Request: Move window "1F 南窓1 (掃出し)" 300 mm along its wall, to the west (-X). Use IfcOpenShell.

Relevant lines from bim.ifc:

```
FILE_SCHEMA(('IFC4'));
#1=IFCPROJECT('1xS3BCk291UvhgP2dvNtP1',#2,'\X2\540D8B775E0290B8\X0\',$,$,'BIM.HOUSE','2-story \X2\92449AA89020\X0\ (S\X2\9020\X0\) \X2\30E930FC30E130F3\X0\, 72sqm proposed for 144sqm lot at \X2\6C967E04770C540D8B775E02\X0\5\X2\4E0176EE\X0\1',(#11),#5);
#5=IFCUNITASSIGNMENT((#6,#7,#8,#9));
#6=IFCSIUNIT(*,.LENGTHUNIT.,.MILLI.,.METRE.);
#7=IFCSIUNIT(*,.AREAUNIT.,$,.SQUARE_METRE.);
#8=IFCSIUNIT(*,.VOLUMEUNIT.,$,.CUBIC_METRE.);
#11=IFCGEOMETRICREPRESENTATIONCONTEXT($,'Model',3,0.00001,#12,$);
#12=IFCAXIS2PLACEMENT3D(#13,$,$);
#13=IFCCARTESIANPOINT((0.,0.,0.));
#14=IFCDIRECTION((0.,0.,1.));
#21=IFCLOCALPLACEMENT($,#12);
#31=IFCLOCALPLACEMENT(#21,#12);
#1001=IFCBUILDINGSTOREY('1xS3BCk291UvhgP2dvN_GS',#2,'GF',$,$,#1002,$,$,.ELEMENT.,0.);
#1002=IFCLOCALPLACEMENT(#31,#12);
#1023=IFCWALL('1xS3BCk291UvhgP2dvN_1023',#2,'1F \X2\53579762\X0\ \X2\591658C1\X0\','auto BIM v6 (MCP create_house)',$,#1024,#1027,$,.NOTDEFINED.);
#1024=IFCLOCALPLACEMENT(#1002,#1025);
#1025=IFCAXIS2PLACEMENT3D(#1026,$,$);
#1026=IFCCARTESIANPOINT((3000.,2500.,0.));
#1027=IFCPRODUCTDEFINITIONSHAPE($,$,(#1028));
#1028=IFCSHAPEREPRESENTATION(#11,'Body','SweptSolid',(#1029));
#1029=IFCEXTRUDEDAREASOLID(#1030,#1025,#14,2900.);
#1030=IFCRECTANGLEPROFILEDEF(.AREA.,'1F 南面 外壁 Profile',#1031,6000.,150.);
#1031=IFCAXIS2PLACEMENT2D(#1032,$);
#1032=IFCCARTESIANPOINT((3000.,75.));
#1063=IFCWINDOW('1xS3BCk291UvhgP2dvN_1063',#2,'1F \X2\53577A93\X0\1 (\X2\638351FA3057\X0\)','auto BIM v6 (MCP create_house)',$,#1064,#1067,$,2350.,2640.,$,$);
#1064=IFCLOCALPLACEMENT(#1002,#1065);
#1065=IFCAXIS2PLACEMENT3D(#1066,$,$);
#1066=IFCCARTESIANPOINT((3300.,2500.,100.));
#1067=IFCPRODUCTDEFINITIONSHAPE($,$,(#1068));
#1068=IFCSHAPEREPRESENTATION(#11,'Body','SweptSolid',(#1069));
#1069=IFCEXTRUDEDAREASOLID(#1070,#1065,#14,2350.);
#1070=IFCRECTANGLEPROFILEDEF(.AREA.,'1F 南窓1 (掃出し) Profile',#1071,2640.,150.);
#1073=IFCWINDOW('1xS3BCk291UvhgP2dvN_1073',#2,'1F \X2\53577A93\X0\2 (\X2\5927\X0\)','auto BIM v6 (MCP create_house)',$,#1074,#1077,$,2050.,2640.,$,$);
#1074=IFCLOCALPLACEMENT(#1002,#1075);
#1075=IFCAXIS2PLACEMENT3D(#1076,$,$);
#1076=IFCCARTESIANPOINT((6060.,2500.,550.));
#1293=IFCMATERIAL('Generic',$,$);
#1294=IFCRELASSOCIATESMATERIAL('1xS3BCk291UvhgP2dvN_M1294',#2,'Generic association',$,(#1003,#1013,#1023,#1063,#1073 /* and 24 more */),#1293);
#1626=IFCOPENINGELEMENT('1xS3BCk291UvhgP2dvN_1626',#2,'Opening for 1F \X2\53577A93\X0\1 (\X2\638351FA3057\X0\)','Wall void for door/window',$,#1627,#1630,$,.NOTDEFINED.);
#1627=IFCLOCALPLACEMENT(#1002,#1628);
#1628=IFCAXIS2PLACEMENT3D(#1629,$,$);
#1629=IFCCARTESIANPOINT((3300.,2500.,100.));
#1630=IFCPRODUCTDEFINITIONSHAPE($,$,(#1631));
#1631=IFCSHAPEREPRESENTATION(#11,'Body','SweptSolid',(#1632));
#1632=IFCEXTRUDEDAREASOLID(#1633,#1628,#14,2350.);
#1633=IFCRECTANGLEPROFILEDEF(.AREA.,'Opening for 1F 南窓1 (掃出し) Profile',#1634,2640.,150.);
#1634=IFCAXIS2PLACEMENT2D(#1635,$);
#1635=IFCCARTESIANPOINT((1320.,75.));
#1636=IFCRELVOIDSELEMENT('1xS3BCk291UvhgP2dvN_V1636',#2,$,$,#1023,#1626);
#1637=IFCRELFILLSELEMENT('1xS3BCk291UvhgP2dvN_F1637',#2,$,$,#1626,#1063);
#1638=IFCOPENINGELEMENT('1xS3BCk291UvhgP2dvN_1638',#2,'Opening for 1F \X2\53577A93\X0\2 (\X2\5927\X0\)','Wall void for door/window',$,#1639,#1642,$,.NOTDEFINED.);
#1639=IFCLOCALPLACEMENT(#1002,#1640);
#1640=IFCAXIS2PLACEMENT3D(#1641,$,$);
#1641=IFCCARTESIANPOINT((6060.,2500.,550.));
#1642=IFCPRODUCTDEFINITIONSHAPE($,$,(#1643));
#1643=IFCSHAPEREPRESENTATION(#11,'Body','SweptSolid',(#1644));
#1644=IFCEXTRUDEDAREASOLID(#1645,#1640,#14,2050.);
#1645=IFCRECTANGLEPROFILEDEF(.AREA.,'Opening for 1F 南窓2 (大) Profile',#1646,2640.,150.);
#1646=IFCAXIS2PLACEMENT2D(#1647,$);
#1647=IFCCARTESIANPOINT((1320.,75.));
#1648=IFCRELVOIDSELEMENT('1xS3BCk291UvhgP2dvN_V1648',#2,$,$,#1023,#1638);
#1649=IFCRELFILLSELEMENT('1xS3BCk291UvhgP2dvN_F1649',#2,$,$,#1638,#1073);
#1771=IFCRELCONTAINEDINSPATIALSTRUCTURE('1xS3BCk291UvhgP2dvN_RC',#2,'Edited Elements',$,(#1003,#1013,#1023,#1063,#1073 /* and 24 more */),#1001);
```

```python
import ifcopenshell
import ifcopenshell.api.geometry
import ifcopenshell.util.placement

model = ifcopenshell.open("bim.ifc")

window = model.by_id(1063)
opening = window.FillsVoids[0].RelatingOpeningElement
wall = opening.VoidsElements[0].RelatingBuildingElement

wall_matrix = ifcopenshell.util.placement.get_local_placement(wall.ObjectPlacement)
shift = wall_matrix[:3, 0] * -300.0
before = ifcopenshell.util.placement.get_local_placement(window.ObjectPlacement)[:3, 3].copy()

# The window is not placed relative to its opening, so move both.
for product in (opening, window):
    matrix = ifcopenshell.util.placement.get_local_placement(product.ObjectPlacement)
    matrix[:3, 3] += shift
    ifcopenshell.api.geometry.edit_object_placement(model, product=product, matrix=matrix, is_si=False)

after = ifcopenshell.util.placement.get_local_placement(window.ObjectPlacement)[:3, 3]
print("window moved by", (after - before).round(3) + 0.0)

model.write("bim_updated.ifc")
```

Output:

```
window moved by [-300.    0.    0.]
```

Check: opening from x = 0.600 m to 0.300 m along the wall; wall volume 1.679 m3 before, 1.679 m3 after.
